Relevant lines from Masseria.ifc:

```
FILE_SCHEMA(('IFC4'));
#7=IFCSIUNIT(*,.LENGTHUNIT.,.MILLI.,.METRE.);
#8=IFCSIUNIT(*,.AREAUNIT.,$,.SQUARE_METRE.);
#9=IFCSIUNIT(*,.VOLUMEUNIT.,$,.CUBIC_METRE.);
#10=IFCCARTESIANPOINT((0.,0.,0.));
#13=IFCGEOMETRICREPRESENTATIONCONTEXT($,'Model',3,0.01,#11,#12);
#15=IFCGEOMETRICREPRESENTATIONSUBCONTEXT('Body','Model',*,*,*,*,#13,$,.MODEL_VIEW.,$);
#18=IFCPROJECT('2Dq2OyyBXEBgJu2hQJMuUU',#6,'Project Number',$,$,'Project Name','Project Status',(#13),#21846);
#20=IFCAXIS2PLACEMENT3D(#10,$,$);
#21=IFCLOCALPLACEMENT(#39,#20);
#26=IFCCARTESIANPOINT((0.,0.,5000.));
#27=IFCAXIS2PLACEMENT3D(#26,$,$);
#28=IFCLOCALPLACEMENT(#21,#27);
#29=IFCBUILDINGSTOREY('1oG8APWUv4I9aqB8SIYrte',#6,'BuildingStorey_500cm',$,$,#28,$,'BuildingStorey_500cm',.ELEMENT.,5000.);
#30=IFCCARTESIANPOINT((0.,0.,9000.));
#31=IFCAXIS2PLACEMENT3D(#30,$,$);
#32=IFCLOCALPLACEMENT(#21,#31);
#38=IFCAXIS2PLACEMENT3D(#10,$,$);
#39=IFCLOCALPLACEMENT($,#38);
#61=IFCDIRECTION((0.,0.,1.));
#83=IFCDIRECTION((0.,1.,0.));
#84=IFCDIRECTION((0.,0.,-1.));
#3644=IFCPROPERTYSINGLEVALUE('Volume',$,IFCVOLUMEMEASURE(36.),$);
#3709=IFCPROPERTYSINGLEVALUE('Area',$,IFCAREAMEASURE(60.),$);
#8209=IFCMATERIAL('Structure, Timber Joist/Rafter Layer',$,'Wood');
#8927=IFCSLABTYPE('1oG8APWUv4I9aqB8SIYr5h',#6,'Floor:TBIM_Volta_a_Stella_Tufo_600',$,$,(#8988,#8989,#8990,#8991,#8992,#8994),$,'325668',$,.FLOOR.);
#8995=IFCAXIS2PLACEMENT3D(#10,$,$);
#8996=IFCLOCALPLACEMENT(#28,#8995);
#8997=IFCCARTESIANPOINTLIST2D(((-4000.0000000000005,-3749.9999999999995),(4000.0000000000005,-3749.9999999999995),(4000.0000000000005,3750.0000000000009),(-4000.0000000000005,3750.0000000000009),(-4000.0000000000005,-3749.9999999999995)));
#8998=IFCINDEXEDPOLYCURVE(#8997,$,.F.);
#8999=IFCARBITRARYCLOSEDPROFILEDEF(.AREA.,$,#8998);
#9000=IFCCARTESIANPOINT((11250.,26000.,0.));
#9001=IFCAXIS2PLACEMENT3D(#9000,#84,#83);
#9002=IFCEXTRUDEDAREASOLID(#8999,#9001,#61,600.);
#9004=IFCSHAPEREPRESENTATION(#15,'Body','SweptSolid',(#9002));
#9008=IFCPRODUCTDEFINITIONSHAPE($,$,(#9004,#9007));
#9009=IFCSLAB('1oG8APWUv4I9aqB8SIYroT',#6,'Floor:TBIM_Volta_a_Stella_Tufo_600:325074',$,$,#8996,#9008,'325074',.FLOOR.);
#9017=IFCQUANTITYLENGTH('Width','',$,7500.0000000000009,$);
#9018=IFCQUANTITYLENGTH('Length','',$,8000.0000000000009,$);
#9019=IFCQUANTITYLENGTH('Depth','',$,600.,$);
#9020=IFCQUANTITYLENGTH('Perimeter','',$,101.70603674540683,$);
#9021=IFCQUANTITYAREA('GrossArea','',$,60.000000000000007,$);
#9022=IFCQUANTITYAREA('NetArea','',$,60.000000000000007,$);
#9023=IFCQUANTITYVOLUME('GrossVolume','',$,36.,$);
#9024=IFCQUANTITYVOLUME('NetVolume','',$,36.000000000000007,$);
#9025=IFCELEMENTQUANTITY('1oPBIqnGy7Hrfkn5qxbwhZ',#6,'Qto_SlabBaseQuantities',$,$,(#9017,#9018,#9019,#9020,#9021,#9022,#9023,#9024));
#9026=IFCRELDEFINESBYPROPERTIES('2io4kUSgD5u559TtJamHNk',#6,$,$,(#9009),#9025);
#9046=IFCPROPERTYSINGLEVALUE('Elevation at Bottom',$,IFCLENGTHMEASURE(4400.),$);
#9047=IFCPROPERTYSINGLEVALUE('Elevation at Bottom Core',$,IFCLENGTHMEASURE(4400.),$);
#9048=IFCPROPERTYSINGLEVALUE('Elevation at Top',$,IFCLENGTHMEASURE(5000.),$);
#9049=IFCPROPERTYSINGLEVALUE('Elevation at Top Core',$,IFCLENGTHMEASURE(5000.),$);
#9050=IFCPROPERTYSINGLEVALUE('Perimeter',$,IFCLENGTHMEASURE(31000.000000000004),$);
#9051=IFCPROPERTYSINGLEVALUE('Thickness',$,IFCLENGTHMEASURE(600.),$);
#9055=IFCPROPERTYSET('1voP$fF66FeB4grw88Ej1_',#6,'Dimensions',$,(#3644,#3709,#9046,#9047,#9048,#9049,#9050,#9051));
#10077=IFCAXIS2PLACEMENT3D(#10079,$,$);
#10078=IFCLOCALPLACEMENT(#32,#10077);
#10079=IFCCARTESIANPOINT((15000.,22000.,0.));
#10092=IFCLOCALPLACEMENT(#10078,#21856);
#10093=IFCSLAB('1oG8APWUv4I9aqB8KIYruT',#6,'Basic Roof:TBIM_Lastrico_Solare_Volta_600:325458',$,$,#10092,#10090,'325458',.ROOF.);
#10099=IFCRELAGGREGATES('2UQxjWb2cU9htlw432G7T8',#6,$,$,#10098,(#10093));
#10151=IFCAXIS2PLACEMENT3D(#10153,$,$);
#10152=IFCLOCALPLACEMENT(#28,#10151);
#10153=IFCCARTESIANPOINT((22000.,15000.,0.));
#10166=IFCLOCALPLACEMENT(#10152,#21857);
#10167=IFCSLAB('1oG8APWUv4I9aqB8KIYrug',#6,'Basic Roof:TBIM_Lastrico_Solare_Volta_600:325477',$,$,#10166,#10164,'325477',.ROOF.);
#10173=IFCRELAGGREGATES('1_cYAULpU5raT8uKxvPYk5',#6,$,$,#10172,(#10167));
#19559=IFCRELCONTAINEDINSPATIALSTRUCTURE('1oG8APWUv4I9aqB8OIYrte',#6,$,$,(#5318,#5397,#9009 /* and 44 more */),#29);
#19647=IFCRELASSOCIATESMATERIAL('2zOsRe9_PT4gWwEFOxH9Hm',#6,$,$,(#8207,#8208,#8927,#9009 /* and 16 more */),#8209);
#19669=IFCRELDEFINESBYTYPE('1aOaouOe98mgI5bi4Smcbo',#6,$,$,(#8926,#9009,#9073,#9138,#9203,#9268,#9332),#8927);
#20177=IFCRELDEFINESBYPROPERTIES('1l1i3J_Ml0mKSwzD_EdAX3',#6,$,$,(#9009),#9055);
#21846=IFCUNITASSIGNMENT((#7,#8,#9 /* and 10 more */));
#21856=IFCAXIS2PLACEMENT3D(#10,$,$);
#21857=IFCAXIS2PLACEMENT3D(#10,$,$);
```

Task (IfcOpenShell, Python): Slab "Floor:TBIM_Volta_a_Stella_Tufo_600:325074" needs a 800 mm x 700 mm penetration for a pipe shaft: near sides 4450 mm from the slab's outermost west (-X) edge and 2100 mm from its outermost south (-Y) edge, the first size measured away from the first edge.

```python
import numpy as np
import ifcopenshell
import ifcopenshell.api.feature
import ifcopenshell.api.geometry
import ifcopenshell.api.pset
import ifcopenshell.api.root
import ifcopenshell.geom
import ifcopenshell.util.element
import ifcopenshell.util.placement
import ifcopenshell.util.representation
import ifcopenshell.util.shape
import ifcopenshell.util.unit

model = ifcopenshell.open("Masseria.ifc")
unit_scale = ifcopenshell.util.unit.calculate_unit_scale(model)
area_scale = ifcopenshell.util.unit.calculate_unit_scale(model, "AREAUNIT")
volume_scale = ifcopenshell.util.unit.calculate_unit_scale(model, "VOLUMEUNIT")
settings = ifcopenshell.geom.settings()


def volume(element):
    """Net volume in cubic metres, openings subtracted."""
    shape = ifcopenshell.geom.create_shape(settings, element)
    return ifcopenshell.util.shape.get_volume(shape.geometry)


slab = model.by_guid("1oG8APWUv4I9aqB8SIYroT")
before = volume(slab)

# Extent in the slab's own axes, in metres. The edges named are its -X and -Y sides.
slab_shape = ifcopenshell.geom.create_shape(settings, slab)
vertices = ifcopenshell.util.shape.get_vertices(slab_shape.geometry)
x_min, y_min, bottom = vertices.min(axis=0)
top = vertices[:, 2].max()

opening = ifcopenshell.api.root.create_entity(model, ifc_class="IfcOpeningElement", name="Pipe shaft opening", predefined_type="OPENING")
context = ifcopenshell.util.representation.get_context(model, "Model", "Body", "MODEL_VIEW")
width, depth = 0.8, 0.7
outline = [(0.0, 0.0), (width, 0.0), (width, depth), (0.0, depth), (0.0, 0.0)]
# Overshoot both faces by 50 mm so the cut is clean.
shape = ifcopenshell.api.geometry.add_slab_representation(
    model, context=context, depth=top - bottom + 0.1, polyline=outline
)
ifcopenshell.api.geometry.assign_representation(model, product=opening, representation=shape)

matrix = ifcopenshell.util.placement.get_local_placement(slab.ObjectPlacement)
matrix[:, 3] = matrix @ np.append(np.array([x_min + 4.45, y_min + 2.1, bottom - 0.05]) / unit_scale, 1.0)
ifcopenshell.api.geometry.edit_object_placement(model, product=opening, matrix=matrix, is_si=False)
ifcopenshell.api.feature.add_feature(model, feature=opening, element=slab)

after = volume(slab)

# Update the slab's stored quantities.
qto = model.by_id(ifcopenshell.util.element.get_pset(slab, "Qto_SlabBaseQuantities", should_inherit=False)["id"])
ifcopenshell.api.pset.edit_qto(model, qto=qto, properties={
    "NetArea": after / (top - bottom) / area_scale,
    "NetVolume": after / volume_scale,
})
pset = model.by_id(ifcopenshell.util.element.get_pset(slab, "Dimensions", should_inherit=False)["id"])
ifcopenshell.api.pset.edit_pset(model, pset=pset, properties={
    "Volume": model.create_entity("IfcVolumeMeasure", after / volume_scale),
    "Area": model.create_entity("IfcAreaMeasure", after / (top - bottom) / area_scale),
})

print(f"slab volume {before:.3f} -> {after:.3f} m3")

model.write("Masseria_edited.ifc")
```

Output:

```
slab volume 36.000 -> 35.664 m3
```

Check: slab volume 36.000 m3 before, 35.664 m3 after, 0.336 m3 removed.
